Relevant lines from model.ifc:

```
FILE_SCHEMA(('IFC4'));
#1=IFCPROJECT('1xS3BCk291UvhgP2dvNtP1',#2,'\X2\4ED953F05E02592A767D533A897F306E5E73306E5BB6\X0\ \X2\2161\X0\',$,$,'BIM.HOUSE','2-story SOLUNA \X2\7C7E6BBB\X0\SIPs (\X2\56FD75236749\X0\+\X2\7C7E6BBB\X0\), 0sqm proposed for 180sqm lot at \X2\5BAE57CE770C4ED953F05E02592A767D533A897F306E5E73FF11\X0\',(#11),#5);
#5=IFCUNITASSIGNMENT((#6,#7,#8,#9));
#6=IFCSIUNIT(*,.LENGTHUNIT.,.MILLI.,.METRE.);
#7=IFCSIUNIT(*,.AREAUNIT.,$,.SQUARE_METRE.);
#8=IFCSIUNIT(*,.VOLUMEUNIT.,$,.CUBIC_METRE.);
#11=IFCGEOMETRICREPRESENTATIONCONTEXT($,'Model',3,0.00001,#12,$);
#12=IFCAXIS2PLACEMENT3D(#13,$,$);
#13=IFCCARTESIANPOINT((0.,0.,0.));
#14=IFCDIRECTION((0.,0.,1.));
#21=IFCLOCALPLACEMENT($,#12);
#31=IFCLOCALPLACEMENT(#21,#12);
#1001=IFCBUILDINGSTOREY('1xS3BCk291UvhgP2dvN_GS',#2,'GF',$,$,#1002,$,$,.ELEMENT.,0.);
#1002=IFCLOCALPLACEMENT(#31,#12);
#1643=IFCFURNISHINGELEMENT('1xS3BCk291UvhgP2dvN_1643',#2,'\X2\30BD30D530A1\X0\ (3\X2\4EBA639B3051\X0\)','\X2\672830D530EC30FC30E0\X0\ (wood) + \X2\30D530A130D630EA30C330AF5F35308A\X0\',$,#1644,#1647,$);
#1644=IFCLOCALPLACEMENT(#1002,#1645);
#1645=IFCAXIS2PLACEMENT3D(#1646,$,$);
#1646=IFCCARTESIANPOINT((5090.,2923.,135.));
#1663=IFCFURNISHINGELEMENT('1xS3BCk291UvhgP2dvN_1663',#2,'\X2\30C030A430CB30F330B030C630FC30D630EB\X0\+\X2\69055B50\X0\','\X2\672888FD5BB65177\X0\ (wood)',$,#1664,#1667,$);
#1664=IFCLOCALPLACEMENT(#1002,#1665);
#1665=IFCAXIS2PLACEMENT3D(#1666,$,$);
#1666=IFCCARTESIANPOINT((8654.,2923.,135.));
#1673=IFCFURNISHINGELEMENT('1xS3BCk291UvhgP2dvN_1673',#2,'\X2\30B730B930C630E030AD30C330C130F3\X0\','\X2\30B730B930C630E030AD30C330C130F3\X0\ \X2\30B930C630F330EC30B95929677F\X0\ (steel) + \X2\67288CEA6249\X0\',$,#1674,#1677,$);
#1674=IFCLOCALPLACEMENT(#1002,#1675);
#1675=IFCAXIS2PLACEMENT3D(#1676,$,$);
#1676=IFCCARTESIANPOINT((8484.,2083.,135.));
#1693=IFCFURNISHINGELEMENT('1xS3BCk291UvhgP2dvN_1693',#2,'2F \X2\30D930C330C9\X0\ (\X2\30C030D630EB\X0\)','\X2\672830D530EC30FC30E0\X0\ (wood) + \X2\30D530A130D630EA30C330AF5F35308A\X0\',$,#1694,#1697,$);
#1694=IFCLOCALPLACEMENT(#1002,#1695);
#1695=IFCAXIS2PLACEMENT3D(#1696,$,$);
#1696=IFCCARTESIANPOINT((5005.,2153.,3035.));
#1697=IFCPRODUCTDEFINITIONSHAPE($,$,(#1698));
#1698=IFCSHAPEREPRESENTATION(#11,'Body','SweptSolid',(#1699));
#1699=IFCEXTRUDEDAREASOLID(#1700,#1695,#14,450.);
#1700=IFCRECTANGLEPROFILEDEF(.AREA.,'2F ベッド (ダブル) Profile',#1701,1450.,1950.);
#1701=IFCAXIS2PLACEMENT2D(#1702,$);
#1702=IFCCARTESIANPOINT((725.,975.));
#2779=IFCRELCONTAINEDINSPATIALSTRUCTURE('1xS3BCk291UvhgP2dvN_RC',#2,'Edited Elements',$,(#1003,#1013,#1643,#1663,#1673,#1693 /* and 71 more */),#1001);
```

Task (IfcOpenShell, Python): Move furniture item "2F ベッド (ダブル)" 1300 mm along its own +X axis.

```python
import ifcopenshell
import ifcopenshell.api.geometry
import ifcopenshell.util.placement
import ifcopenshell.util.unit

model = ifcopenshell.open("model.ifc")
unit_scale = ifcopenshell.util.unit.calculate_unit_scale(model)

item = model.by_guid("1xS3BCk291UvhgP2dvN_1693")
matrix = ifcopenshell.util.placement.get_local_placement(item.ObjectPlacement)
matrix[:3, 3] += matrix[:3, 0] * 1.3 / unit_scale
ifcopenshell.api.geometry.edit_object_placement(model, product=item, matrix=matrix, is_si=False)

print(ifcopenshell.util.placement.get_local_placement(item.ObjectPlacement).round(3) + 0.0)

model.write("model_rev.ifc")
```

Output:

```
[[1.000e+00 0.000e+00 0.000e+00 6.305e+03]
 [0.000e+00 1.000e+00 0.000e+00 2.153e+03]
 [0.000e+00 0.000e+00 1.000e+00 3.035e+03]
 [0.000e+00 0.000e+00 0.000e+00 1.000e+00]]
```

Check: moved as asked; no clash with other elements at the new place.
